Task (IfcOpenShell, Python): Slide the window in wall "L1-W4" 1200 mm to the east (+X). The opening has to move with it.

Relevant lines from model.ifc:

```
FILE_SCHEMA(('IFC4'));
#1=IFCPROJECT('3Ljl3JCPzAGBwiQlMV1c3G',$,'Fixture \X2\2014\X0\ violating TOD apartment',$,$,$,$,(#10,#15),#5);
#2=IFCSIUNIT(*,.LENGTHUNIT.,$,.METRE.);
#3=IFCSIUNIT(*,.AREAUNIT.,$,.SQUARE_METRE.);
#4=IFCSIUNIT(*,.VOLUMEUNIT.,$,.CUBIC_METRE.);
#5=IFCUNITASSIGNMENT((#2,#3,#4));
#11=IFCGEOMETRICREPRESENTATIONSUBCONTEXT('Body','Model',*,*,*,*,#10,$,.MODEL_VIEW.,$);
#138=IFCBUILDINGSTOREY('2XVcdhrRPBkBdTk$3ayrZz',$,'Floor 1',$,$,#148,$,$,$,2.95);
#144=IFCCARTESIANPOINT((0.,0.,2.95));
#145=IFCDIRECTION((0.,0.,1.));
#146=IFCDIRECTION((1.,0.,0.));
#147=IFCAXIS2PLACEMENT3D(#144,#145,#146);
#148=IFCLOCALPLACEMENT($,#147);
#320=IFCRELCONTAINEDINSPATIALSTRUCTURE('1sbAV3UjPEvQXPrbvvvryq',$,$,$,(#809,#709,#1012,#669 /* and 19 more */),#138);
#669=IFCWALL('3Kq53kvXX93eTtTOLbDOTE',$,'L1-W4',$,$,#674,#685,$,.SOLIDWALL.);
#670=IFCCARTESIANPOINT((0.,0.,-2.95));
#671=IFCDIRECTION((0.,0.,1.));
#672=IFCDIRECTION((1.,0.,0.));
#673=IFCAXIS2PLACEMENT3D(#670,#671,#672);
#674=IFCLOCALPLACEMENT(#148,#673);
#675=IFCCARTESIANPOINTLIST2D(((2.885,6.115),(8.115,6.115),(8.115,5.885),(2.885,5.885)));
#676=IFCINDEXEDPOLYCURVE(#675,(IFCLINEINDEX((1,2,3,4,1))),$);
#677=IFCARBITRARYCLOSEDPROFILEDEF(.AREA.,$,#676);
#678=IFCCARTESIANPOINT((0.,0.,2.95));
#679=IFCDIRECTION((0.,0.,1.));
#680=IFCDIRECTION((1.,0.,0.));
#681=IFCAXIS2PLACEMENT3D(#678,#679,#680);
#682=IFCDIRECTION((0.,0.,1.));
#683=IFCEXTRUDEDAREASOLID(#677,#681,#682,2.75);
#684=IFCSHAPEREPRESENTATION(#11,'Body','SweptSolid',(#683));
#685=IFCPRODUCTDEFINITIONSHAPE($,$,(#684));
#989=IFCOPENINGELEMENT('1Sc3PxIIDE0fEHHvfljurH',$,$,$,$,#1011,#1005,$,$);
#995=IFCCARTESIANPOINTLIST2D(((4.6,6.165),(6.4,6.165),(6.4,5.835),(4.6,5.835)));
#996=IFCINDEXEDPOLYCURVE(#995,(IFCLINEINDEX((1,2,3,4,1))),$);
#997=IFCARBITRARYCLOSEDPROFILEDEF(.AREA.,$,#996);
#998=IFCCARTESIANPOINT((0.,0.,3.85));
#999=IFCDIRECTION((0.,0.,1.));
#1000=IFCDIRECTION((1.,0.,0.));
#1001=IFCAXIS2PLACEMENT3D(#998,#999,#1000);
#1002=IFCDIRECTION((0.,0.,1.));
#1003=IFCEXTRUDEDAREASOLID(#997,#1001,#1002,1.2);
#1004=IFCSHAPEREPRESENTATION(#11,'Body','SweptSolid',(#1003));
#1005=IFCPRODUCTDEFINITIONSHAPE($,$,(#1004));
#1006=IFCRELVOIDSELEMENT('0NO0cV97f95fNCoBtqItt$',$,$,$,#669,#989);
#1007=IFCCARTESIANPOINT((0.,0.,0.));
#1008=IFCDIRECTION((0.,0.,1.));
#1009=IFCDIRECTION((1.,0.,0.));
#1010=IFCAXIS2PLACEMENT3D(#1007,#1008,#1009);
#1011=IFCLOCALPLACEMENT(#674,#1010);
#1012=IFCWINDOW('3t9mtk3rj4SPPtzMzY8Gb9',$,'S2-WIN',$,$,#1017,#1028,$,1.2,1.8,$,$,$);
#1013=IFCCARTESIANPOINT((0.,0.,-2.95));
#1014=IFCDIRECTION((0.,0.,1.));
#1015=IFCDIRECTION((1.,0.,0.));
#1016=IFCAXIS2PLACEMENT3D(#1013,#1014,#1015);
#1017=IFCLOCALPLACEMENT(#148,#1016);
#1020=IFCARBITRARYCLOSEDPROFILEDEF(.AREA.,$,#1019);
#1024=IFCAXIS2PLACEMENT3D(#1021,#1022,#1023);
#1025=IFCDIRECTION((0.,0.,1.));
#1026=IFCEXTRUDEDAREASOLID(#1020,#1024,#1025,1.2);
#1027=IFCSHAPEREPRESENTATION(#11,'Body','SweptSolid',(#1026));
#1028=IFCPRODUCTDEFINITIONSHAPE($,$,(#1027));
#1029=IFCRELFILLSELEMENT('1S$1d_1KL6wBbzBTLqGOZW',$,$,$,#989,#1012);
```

```python
import ifcopenshell
import ifcopenshell.api.geometry
import ifcopenshell.util.placement
import ifcopenshell.util.unit

model = ifcopenshell.open("model.ifc")
unit_scale = ifcopenshell.util.unit.calculate_unit_scale(model)

window = model.by_id(1012)
opening = window.FillsVoids[0].RelatingOpeningElement
wall = opening.VoidsElements[0].RelatingBuildingElement

wall_matrix = ifcopenshell.util.placement.get_local_placement(wall.ObjectPlacement)
shift = wall_matrix[:3, 0] * 1.2 / unit_scale
before = ifcopenshell.util.placement.get_local_placement(window.ObjectPlacement)[:3, 3].copy()

# The window is not placed relative to its opening, so move both.
for product in (opening, window):
    matrix = ifcopenshell.util.placement.get_local_placement(product.ObjectPlacement)
    matrix[:3, 3] += shift
    ifcopenshell.api.geometry.edit_object_placement(model, product=product, matrix=matrix, is_si=False)

after = ifcopenshell.util.placement.get_local_placement(window.ObjectPlacement)[:3, 3]
print("window moved by", (after - before).round(3) + 0.0)

model.write("model-out.ifc")
```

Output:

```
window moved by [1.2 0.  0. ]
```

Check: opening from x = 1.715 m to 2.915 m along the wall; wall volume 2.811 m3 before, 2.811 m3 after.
